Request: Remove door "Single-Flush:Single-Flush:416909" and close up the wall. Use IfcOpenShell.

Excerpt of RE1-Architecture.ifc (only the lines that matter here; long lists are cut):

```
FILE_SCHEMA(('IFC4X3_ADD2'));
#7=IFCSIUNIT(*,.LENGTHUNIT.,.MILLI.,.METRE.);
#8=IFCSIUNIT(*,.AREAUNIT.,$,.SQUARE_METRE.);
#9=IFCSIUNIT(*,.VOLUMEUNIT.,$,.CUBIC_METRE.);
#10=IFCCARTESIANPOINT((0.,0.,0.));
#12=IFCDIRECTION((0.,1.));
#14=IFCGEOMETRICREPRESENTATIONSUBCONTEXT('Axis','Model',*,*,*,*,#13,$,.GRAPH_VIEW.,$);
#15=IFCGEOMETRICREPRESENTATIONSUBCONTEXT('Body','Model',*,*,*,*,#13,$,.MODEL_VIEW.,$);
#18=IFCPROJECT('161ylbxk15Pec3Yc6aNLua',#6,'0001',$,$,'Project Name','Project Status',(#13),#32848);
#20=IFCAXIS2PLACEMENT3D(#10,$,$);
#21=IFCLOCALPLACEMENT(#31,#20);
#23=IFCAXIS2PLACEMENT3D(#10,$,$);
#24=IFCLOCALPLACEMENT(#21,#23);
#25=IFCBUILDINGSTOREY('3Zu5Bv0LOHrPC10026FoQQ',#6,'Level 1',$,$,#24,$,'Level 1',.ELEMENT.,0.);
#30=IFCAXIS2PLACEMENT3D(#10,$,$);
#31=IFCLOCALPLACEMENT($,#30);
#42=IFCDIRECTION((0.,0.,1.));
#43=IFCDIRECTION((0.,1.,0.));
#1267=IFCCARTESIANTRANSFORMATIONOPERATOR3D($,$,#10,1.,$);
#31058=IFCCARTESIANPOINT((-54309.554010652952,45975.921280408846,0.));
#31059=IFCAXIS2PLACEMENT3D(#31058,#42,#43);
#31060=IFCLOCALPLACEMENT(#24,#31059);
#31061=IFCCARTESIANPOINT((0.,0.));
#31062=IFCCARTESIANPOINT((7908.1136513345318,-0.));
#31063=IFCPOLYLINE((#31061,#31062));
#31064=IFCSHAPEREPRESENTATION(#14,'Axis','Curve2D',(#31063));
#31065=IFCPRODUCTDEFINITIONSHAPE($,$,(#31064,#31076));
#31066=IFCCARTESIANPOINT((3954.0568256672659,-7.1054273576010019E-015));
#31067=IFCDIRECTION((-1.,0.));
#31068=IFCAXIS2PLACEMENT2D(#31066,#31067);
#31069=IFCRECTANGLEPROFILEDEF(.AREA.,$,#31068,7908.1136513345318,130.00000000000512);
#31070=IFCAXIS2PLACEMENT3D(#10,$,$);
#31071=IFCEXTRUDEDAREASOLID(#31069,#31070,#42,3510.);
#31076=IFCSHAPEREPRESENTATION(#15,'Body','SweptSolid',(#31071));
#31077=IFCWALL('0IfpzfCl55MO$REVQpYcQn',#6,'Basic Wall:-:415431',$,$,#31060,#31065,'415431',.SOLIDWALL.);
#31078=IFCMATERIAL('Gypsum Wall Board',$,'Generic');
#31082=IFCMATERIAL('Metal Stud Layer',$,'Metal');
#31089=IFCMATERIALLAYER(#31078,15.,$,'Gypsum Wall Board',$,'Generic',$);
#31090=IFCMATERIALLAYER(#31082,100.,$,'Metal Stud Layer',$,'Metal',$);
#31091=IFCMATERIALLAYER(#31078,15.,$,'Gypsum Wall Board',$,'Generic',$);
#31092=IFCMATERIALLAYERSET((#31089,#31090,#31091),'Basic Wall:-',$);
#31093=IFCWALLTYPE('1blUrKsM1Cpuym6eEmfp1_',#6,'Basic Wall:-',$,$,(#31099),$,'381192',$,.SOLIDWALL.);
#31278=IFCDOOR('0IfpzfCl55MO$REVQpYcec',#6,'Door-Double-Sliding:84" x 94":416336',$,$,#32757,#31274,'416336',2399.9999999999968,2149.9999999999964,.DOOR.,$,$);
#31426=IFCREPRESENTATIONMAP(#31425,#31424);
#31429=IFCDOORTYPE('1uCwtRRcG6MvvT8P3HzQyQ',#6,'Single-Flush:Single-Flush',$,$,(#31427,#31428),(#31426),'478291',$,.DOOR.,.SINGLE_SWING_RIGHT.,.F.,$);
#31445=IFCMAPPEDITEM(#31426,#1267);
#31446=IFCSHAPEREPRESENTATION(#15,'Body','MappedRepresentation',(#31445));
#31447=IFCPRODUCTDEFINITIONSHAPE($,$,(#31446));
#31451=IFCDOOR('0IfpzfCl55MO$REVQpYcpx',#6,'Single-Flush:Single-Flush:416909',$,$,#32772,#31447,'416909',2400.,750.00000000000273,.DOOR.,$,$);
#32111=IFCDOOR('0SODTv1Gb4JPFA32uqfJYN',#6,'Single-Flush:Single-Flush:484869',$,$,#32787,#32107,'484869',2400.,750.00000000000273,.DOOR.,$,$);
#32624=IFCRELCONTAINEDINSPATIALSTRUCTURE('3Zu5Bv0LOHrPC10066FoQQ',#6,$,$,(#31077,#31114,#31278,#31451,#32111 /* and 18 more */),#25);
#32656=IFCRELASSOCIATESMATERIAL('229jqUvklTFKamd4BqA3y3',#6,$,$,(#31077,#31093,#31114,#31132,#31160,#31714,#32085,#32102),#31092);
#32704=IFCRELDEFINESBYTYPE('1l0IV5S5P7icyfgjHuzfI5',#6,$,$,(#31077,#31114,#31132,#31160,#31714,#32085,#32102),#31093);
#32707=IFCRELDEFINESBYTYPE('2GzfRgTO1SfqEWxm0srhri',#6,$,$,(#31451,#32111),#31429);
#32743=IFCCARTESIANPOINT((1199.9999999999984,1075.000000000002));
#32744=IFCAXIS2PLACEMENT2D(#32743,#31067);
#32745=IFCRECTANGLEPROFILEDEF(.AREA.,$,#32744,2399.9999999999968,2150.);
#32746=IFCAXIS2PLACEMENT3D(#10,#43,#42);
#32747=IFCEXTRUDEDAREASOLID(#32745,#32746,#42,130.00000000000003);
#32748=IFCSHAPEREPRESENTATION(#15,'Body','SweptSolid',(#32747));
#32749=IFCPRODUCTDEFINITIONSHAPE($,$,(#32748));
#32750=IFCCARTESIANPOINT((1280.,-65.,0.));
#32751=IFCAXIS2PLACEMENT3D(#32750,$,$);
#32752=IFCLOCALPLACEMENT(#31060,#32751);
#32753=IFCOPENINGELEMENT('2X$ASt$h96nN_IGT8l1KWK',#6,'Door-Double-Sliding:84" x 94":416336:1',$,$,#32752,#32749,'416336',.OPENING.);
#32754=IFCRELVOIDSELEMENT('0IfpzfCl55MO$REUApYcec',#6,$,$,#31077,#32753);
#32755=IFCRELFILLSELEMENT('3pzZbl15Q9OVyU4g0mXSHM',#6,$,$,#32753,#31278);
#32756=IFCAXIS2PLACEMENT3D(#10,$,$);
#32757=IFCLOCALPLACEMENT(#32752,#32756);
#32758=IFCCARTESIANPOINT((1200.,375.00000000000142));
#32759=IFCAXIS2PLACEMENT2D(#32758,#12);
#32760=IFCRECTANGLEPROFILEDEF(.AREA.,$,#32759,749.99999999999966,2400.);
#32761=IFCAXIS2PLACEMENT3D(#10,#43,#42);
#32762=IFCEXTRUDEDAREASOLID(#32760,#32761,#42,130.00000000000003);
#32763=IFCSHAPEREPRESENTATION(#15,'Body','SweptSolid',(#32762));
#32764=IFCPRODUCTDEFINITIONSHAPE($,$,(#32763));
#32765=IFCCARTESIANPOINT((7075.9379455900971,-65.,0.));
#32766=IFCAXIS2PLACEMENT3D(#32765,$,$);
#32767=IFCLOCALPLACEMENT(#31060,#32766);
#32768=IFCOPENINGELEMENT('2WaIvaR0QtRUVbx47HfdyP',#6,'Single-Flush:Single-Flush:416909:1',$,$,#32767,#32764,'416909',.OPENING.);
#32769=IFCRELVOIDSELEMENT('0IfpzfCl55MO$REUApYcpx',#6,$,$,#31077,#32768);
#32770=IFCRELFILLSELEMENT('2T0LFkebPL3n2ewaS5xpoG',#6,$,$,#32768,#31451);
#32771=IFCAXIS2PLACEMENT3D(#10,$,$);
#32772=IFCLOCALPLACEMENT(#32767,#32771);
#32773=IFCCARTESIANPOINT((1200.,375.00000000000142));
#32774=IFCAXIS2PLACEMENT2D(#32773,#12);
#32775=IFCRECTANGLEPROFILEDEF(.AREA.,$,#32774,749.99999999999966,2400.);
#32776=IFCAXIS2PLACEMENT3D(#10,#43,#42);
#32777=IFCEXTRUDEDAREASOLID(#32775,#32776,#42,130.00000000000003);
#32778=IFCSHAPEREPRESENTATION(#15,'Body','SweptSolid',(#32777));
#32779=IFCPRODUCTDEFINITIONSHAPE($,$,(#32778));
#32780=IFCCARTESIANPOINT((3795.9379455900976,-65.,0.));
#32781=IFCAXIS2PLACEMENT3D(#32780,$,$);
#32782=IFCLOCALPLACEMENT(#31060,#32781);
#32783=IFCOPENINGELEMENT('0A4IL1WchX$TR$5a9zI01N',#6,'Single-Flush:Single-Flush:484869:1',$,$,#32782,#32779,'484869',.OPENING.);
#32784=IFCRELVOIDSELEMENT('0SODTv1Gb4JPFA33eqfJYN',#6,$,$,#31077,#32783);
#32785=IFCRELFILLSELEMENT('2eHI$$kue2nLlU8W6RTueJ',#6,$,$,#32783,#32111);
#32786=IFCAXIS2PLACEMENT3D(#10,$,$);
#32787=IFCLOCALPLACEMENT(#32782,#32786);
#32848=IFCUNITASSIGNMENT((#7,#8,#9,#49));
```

```python
import ifcopenshell
import ifcopenshell.api.feature
import ifcopenshell.api.root
import ifcopenshell.geom
import ifcopenshell.util.shape

model = ifcopenshell.open("RE1-Architecture.ifc")
settings = ifcopenshell.geom.settings()


def volume(element):
    """Net volume in cubic metres, openings subtracted."""
    shape = ifcopenshell.geom.create_shape(settings, element)
    return ifcopenshell.util.shape.get_volume(shape.geometry)


door = model.by_guid("0IfpzfCl55MO$REVQpYcpx")
opening = door.FillsVoids[0].RelatingOpeningElement
wall = opening.VoidsElements[0].RelatingBuildingElement
before = volume(wall)

ifcopenshell.api.root.remove_product(model, product=door)
ifcopenshell.api.feature.remove_feature(model, feature=opening)

after = volume(wall)

print(f"wall volume {before:.3f} -> {after:.3f} m3")

model.write("RE1-Architecture_updated.ifc")
```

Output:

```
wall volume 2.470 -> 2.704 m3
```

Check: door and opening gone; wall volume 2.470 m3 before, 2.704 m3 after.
